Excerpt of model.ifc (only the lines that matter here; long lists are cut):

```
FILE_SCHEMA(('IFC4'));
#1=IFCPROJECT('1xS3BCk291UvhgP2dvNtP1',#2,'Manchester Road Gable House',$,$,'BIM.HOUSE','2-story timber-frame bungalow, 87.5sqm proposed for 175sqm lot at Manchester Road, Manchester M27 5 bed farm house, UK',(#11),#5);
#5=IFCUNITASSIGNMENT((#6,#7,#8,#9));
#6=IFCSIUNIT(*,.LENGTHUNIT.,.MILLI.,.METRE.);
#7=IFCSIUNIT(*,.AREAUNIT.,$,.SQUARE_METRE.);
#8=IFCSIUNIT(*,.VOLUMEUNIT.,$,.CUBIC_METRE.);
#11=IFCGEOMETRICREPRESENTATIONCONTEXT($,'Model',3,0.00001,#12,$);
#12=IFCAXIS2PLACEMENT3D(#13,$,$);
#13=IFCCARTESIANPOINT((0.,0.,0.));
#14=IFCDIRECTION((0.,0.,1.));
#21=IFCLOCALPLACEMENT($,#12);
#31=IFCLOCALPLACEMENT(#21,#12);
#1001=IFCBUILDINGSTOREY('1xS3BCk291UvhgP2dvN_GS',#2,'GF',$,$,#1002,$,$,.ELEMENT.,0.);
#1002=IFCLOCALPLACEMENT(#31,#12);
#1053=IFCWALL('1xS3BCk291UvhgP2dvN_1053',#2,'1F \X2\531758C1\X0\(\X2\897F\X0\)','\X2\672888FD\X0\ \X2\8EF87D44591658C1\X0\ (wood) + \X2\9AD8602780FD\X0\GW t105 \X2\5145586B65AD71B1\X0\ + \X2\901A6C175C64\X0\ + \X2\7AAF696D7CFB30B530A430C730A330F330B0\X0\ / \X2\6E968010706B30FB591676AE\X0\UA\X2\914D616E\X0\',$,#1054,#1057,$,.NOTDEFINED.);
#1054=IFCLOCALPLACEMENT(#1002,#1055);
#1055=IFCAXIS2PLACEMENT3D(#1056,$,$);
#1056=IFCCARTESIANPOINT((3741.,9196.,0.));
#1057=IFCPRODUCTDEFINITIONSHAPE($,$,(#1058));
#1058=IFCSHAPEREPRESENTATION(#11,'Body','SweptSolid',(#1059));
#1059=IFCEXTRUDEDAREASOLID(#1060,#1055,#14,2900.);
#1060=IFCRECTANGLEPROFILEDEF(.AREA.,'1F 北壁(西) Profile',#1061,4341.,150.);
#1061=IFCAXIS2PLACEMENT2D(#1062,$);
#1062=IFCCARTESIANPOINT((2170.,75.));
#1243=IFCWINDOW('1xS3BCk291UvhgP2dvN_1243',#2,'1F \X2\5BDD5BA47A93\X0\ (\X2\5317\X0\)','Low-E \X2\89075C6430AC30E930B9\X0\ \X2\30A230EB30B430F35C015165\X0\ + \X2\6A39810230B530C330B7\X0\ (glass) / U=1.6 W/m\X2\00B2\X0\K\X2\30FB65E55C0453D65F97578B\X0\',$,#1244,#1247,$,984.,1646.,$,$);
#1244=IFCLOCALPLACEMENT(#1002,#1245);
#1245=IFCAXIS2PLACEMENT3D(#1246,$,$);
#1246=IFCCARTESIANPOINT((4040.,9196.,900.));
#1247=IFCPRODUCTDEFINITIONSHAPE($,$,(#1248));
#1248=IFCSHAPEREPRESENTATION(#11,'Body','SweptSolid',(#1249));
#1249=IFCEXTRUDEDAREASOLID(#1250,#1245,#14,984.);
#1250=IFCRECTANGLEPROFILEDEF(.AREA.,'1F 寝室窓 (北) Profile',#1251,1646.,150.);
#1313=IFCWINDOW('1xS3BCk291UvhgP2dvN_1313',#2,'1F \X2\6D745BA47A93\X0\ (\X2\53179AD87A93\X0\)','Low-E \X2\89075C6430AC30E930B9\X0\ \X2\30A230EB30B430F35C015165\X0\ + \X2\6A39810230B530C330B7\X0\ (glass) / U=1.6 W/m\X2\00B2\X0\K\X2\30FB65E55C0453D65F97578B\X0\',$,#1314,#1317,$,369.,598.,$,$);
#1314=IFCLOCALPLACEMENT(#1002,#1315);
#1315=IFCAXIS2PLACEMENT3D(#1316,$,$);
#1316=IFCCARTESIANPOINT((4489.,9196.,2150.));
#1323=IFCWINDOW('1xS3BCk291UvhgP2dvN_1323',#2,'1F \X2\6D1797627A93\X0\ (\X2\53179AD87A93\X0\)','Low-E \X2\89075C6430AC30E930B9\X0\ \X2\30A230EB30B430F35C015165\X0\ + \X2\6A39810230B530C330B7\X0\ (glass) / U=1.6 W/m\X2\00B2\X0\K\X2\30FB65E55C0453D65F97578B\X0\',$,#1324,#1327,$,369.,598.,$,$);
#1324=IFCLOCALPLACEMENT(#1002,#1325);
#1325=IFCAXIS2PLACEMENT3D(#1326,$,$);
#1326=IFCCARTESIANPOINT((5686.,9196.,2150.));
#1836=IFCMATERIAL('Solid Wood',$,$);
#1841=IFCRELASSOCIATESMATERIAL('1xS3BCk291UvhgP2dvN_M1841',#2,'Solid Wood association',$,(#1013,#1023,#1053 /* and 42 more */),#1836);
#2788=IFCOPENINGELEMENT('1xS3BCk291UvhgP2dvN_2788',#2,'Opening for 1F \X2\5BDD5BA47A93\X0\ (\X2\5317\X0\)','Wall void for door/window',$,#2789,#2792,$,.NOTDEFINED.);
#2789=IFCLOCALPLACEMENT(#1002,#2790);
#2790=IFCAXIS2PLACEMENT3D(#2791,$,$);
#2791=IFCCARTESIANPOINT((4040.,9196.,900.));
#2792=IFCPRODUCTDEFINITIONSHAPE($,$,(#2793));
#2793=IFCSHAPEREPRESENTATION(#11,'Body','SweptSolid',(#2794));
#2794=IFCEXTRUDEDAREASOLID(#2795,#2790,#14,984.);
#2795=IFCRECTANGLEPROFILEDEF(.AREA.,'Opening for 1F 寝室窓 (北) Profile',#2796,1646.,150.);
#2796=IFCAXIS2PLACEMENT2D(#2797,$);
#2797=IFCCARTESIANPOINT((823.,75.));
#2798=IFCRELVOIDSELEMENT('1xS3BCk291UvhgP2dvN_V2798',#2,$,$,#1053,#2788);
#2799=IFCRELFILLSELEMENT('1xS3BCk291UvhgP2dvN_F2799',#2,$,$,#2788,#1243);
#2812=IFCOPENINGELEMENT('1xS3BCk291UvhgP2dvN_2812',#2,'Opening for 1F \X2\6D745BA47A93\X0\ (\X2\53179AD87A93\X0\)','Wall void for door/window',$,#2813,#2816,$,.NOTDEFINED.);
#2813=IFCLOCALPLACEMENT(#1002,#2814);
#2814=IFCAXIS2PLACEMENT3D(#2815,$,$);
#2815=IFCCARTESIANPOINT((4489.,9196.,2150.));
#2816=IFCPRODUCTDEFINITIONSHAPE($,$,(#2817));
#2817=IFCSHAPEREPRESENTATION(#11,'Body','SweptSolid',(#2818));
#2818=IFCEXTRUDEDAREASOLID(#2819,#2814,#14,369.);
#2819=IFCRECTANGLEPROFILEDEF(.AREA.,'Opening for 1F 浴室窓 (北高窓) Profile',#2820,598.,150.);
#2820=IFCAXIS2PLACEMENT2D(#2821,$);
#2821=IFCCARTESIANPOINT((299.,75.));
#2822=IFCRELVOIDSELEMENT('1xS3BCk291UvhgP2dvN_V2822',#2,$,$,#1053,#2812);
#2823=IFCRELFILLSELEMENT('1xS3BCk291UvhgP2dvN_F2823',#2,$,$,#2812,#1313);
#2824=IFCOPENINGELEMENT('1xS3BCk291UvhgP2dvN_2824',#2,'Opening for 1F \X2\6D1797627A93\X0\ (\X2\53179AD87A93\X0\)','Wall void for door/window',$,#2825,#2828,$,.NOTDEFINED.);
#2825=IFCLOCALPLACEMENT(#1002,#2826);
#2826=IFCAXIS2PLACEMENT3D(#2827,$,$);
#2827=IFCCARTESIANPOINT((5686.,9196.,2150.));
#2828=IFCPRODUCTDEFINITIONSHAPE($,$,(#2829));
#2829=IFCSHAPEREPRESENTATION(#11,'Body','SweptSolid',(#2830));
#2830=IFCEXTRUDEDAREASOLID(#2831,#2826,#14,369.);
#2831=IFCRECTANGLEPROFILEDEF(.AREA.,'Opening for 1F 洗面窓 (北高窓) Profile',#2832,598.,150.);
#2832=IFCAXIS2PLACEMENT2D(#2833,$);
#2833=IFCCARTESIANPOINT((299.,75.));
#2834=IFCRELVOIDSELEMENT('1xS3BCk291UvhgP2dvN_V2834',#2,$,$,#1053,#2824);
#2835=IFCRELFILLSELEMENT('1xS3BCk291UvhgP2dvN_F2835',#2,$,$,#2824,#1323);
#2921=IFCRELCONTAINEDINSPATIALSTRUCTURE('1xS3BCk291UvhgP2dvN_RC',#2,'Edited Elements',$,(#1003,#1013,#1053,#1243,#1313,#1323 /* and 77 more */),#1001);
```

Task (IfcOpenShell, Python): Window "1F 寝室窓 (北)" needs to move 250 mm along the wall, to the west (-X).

```python
import ifcopenshell
import ifcopenshell.api.geometry
import ifcopenshell.util.placement

model = ifcopenshell.open("model.ifc")

window = model.by_id(1243)
opening = window.FillsVoids[0].RelatingOpeningElement
wall = opening.VoidsElements[0].RelatingBuildingElement

wall_matrix = ifcopenshell.util.placement.get_local_placement(wall.ObjectPlacement)
shift = wall_matrix[:3, 0] * -250.0
before = ifcopenshell.util.placement.get_local_placement(window.ObjectPlacement)[:3, 3].copy()

# The window is not placed relative to its opening, so move both.
for product in (opening, window):
    matrix = ifcopenshell.util.placement.get_local_placement(product.ObjectPlacement)
    matrix[:3, 3] += shift
    ifcopenshell.api.geometry.edit_object_placement(model, product=product, matrix=matrix, is_si=False)

after = ifcopenshell.util.placement.get_local_placement(window.ObjectPlacement)[:3, 3]
print("window moved by", (after - before).round(3) + 0.0)

model.write("model_v2.ifc")
```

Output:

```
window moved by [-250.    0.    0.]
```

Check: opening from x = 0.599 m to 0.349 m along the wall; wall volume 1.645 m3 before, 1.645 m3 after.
